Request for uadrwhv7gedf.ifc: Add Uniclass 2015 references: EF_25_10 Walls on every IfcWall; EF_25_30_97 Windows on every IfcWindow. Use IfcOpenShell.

First a look at what the model holds.

```python
import ifcopenshell

model = ifcopenshell.open("uadrwhv7gedf.ifc")
print(model.schema)
print("classifications:", [c.Name for c in model.by_type("IfcClassification")])
for ifc_class in ("IfcDoor", "IfcRoof", "IfcStair", "IfcWall", "IfcWindow"):
    print(ifc_class, len(model.by_type(ifc_class)))
```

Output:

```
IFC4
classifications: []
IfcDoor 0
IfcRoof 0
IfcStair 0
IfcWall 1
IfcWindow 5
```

```python
import ifcopenshell
import ifcopenshell.api.classification

model = ifcopenshell.open("uadrwhv7gedf.ifc")

system = ifcopenshell.api.classification.add_classification(model, classification="Uniclass 2015")

codes = {
    "IfcWall": ("EF_25_10", "Walls"),
    "IfcWindow": ("EF_25_30_97", "Windows"),
}
for ifc_class, (code, name) in codes.items():
    products = model.by_type(ifc_class)
    ifcopenshell.api.classification.add_reference(
        model, products=products, classification=system, identification=code, name=name
    )
    print(code, len(products))

model.write("uadrwhv7gedf-out.ifc")
```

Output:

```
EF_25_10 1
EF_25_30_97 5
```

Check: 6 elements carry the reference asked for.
